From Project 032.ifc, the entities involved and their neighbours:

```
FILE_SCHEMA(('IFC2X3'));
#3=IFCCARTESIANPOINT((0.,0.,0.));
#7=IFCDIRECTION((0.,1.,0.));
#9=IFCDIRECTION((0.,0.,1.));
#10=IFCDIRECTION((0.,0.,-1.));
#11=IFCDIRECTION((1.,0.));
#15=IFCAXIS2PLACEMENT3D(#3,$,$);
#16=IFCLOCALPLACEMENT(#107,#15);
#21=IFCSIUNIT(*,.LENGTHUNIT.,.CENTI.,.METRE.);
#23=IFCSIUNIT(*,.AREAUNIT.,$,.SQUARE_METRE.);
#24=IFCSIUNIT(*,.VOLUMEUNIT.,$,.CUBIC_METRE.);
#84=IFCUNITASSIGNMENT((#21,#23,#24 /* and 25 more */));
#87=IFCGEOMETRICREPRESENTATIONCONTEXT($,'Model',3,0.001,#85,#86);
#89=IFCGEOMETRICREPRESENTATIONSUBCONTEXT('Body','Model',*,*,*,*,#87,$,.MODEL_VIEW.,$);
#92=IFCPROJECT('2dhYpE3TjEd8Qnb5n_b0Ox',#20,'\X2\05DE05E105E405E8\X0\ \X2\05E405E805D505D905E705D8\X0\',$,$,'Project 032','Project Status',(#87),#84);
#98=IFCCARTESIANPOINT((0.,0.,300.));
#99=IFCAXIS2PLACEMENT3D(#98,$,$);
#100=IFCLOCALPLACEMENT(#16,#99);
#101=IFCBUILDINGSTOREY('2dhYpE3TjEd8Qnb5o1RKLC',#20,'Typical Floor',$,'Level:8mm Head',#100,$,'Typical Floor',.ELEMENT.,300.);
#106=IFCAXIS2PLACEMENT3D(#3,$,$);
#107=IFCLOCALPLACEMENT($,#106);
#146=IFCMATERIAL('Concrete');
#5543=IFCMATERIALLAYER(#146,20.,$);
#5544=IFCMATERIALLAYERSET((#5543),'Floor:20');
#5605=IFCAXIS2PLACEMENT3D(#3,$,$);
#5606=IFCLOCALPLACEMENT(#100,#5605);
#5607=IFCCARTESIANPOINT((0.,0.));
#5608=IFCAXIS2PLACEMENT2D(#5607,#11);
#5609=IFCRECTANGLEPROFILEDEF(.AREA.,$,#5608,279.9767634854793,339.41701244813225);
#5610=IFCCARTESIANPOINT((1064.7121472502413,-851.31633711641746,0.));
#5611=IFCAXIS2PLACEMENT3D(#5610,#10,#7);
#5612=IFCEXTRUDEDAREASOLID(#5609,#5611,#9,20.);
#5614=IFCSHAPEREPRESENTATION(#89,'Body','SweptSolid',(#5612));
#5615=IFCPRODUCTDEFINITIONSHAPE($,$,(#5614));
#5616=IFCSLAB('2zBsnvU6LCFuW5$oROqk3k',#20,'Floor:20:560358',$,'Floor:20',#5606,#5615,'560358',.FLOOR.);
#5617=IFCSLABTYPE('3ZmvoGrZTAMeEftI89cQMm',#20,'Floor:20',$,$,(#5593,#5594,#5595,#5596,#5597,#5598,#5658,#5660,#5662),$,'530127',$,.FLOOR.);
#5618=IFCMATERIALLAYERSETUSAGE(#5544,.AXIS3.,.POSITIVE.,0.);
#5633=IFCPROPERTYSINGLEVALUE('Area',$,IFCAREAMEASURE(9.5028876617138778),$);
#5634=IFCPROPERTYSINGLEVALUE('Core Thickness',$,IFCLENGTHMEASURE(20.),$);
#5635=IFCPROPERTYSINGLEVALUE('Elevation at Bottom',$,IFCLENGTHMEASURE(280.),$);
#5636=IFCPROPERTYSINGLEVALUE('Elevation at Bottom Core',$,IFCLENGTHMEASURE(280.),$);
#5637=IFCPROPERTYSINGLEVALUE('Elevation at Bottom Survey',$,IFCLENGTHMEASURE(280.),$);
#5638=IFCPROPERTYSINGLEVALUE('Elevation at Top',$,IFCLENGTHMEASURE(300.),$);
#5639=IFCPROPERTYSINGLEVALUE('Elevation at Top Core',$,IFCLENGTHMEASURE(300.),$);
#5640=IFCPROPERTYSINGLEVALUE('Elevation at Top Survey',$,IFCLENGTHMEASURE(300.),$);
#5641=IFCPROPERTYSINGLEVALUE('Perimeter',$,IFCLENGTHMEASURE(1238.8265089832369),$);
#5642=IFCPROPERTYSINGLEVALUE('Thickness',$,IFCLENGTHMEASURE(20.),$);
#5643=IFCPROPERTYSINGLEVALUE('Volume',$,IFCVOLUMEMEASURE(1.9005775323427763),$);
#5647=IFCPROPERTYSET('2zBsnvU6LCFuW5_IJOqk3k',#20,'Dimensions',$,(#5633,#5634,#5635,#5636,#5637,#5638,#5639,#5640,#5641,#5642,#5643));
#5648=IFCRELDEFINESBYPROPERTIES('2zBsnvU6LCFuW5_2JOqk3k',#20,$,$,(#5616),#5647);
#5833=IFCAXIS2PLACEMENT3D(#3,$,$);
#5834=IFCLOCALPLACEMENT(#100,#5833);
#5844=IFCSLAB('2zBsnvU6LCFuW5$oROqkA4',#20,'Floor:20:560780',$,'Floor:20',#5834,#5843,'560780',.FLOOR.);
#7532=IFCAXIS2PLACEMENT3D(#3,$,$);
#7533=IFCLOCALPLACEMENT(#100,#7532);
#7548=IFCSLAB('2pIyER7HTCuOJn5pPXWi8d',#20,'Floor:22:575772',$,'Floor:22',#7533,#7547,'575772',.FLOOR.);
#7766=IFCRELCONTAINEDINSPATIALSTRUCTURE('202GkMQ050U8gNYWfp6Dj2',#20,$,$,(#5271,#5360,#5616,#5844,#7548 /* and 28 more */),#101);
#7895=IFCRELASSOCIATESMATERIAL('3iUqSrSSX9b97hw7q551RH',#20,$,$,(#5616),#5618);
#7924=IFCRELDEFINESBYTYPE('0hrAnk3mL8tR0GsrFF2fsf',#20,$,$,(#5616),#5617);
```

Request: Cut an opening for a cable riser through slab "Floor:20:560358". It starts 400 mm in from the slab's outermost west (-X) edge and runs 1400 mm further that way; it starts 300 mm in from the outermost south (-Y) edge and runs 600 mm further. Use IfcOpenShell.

```python
import numpy as np
import ifcopenshell
import ifcopenshell.api.feature
import ifcopenshell.api.geometry
import ifcopenshell.api.pset
import ifcopenshell.api.root
import ifcopenshell.geom
import ifcopenshell.util.element
import ifcopenshell.util.placement
import ifcopenshell.util.representation
import ifcopenshell.util.shape
import ifcopenshell.util.unit

model = ifcopenshell.open("Project 032.ifc")
unit_scale = ifcopenshell.util.unit.calculate_unit_scale(model)
area_scale = ifcopenshell.util.unit.calculate_unit_scale(model, "AREAUNIT")
volume_scale = ifcopenshell.util.unit.calculate_unit_scale(model, "VOLUMEUNIT")
settings = ifcopenshell.geom.settings()


def volume(element):
    """Net volume in cubic metres, openings subtracted."""
    shape = ifcopenshell.geom.create_shape(settings, element)
    return ifcopenshell.util.shape.get_volume(shape.geometry)


slab = model.by_guid("2zBsnvU6LCFuW5$oROqk3k")
before = volume(slab)

# Extent in the slab's own axes, in metres. The edges named are its -X and -Y sides.
slab_shape = ifcopenshell.geom.create_shape(settings, slab)
vertices = ifcopenshell.util.shape.get_vertices(slab_shape.geometry)
x_min, y_min, bottom = vertices.min(axis=0)
top = vertices[:, 2].max()

opening = ifcopenshell.api.root.create_entity(model, ifc_class="IfcOpeningElement", name="Cable riser opening")
context = ifcopenshell.util.representation.get_context(model, "Model", "Body", "MODEL_VIEW")
width, depth = 1.4, 0.6
outline = [(0.0, 0.0), (width, 0.0), (width, depth), (0.0, depth), (0.0, 0.0)]
# Overshoot both faces by 50 mm so the cut is clean.
shape = ifcopenshell.api.geometry.add_slab_representation(
    model, context=context, depth=top - bottom + 0.1, polyline=outline
)
ifcopenshell.api.geometry.assign_representation(model, product=opening, representation=shape)

matrix = ifcopenshell.util.placement.get_local_placement(slab.ObjectPlacement)
matrix[:, 3] = matrix @ np.append(np.array([x_min + 0.4, y_min + 0.3, bottom - 0.05]) / unit_scale, 1.0)
ifcopenshell.api.geometry.edit_object_placement(model, product=opening, matrix=matrix, is_si=False)
ifcopenshell.api.feature.add_feature(model, feature=opening, element=slab)

after = volume(slab)

# Update the slab's stored quantities.
pset = model.by_id(ifcopenshell.util.element.get_pset(slab, "Dimensions", should_inherit=False)["id"])
ifcopenshell.api.pset.edit_pset(model, pset=pset, properties={
    "Area": model.create_entity("IfcAreaMeasure", after / (top - bottom) / area_scale),
    "Volume": model.create_entity("IfcVolumeMeasure", after / volume_scale),
})

print(f"slab volume {before:.3f} -> {after:.3f} m3")

model.write("Project 032_edited.ifc")
```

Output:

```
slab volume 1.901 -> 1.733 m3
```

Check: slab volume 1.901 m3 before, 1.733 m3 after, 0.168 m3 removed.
